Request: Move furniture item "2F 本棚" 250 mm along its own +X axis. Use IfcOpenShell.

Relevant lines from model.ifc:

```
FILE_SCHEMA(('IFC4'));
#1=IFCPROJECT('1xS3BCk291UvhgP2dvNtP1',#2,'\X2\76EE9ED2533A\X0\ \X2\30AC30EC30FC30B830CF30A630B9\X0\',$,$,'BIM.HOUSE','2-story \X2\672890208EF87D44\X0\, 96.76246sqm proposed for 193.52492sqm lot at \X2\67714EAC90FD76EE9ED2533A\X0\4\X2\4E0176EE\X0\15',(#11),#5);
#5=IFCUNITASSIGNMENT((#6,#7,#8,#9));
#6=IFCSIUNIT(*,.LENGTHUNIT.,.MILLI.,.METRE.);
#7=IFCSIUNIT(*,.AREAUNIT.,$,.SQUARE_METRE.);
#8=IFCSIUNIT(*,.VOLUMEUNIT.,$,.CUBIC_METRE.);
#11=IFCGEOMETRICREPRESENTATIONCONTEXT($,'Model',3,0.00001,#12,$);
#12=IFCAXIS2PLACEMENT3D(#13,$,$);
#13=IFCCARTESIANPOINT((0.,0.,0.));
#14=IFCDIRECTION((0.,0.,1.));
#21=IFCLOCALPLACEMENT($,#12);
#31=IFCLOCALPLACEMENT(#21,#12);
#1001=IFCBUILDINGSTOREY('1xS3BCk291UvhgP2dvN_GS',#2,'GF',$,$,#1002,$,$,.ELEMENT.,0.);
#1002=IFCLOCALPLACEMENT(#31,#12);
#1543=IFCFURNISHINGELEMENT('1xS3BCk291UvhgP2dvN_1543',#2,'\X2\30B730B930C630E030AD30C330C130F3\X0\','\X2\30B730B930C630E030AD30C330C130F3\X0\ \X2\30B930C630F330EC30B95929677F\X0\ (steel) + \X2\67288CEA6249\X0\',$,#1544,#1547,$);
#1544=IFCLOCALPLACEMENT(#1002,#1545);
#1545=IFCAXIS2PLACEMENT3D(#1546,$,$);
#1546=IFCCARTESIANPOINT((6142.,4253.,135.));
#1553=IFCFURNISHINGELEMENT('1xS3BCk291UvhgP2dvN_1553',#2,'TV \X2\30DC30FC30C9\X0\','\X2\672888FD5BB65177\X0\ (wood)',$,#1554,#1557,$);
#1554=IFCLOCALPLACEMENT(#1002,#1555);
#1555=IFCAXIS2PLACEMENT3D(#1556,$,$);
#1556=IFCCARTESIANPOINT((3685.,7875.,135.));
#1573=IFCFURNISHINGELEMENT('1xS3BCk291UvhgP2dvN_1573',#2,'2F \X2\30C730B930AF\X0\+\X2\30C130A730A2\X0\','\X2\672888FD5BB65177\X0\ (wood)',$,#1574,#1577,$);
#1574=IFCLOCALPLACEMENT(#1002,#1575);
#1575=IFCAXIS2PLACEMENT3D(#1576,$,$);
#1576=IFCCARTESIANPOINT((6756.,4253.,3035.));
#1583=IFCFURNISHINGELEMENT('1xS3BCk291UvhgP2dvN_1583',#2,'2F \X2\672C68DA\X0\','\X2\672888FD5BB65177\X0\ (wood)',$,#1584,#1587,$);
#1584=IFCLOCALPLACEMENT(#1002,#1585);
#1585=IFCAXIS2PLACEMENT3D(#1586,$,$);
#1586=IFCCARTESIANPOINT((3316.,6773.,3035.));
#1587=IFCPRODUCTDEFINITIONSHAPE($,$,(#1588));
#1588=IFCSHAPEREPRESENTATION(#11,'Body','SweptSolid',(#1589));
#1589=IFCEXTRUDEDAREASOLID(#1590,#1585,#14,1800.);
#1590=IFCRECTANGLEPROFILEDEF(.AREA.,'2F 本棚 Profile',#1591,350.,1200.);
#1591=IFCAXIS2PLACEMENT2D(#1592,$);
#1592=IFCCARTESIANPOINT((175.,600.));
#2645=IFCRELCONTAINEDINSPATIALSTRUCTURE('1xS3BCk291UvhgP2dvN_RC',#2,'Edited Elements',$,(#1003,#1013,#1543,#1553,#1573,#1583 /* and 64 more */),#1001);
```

```python
import ifcopenshell
import ifcopenshell.api.geometry
import ifcopenshell.util.placement
import ifcopenshell.util.unit

model = ifcopenshell.open("model.ifc")
unit_scale = ifcopenshell.util.unit.calculate_unit_scale(model)

item = model.by_guid("1xS3BCk291UvhgP2dvN_1583")
matrix = ifcopenshell.util.placement.get_local_placement(item.ObjectPlacement)
matrix[:3, 3] += matrix[:3, 0] * 0.25 / unit_scale
ifcopenshell.api.geometry.edit_object_placement(model, product=item, matrix=matrix, is_si=False)

print(ifcopenshell.util.placement.get_local_placement(item.ObjectPlacement).round(3) + 0.0)

model.write("model-out.ifc")
```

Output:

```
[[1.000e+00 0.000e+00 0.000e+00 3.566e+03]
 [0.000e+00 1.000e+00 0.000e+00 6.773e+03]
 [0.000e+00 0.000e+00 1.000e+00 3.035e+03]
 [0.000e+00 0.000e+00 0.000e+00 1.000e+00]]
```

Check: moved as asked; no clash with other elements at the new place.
